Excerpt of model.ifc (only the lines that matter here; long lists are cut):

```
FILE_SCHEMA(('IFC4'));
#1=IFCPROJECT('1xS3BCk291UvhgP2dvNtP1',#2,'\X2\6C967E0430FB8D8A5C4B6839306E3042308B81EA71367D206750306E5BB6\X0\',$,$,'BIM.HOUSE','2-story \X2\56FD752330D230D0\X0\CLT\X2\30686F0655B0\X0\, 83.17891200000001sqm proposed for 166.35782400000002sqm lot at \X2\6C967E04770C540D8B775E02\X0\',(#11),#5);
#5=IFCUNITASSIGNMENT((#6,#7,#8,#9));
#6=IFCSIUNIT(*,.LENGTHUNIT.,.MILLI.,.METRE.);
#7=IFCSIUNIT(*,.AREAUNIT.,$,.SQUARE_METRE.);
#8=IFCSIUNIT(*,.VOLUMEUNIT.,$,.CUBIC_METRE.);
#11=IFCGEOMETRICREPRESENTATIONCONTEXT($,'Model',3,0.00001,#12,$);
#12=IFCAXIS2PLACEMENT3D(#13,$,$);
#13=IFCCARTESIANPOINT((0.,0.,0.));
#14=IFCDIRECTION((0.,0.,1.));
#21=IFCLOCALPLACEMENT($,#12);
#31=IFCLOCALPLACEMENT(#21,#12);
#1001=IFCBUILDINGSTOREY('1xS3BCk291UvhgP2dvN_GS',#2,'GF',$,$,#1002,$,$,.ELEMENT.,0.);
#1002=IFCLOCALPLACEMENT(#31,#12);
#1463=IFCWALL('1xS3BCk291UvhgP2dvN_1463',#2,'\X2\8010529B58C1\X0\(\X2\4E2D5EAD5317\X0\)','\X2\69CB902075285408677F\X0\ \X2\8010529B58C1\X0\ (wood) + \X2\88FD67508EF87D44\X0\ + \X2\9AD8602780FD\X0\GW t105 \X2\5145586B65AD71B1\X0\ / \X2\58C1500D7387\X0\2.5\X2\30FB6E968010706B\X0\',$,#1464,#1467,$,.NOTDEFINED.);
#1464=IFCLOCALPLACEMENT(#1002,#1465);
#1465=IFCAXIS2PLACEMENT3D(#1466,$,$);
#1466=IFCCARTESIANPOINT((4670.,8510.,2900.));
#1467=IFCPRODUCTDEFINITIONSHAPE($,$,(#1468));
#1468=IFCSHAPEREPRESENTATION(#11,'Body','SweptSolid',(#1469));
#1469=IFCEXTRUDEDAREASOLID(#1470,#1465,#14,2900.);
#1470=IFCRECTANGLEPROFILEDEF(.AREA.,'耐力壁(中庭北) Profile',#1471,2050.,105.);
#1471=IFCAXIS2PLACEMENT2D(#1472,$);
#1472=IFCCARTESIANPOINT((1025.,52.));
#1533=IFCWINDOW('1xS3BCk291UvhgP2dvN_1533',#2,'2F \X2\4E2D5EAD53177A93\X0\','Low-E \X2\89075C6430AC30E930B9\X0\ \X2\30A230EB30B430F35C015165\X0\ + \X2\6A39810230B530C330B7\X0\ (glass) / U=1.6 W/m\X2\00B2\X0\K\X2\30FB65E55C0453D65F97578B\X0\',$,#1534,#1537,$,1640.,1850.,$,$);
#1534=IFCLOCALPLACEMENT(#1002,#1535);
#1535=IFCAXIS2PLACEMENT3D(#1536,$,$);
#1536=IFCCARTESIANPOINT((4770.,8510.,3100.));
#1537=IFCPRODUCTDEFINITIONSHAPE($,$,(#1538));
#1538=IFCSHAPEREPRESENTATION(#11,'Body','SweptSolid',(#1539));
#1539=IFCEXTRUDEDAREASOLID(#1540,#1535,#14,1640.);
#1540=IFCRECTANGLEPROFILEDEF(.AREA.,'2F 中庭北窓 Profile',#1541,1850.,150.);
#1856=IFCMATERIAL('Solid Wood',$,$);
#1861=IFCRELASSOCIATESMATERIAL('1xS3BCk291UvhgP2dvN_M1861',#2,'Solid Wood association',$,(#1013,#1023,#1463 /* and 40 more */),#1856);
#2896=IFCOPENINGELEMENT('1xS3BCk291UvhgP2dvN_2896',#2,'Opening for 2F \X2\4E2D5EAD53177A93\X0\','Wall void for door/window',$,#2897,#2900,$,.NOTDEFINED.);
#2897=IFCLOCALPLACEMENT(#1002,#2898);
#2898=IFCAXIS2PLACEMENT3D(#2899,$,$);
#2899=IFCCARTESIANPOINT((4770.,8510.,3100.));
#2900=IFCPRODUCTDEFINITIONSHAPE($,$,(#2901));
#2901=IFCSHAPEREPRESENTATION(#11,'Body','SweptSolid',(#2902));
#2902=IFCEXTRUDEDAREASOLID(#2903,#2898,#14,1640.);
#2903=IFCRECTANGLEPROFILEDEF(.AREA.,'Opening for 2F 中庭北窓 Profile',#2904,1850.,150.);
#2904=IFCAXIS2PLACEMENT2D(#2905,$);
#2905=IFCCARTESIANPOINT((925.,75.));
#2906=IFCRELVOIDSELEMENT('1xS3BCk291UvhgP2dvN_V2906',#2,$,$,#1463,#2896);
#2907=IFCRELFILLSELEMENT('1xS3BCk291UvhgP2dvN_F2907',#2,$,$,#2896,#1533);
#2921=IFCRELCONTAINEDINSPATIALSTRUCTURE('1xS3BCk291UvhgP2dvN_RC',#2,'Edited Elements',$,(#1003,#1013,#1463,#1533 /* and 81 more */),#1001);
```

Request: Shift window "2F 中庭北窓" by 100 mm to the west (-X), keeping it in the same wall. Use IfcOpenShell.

```python
import ifcopenshell
import ifcopenshell.api.geometry
import ifcopenshell.util.placement
import ifcopenshell.util.unit

model = ifcopenshell.open("model.ifc")
unit_scale = ifcopenshell.util.unit.calculate_unit_scale(model)

window = model.by_guid("1xS3BCk291UvhgP2dvN_1533")
opening = window.FillsVoids[0].RelatingOpeningElement
wall = opening.VoidsElements[0].RelatingBuildingElement

wall_matrix = ifcopenshell.util.placement.get_local_placement(wall.ObjectPlacement)
shift = wall_matrix[:3, 0] * -0.1 / unit_scale
before = ifcopenshell.util.placement.get_local_placement(window.ObjectPlacement)[:3, 3].copy()

# The window is not placed relative to its opening, so move both.
for product in (opening, window):
    matrix = ifcopenshell.util.placement.get_local_placement(product.ObjectPlacement)
    matrix[:3, 3] += shift
    ifcopenshell.api.geometry.edit_object_placement(model, product=product, matrix=matrix, is_si=False)

after = ifcopenshell.util.placement.get_local_placement(window.ObjectPlacement)[:3, 3]
print("window moved by", (after - before).round(3) + 0.0)

model.write("model_edited.ifc")
```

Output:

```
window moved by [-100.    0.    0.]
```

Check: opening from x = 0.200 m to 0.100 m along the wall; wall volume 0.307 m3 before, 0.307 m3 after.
